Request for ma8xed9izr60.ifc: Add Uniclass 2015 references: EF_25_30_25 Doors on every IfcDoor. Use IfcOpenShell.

First a look at what the model holds.

```python
import ifcopenshell

model = ifcopenshell.open("ma8xed9izr60.ifc")
print(model.schema)
print("classifications:", [c.Name for c in model.by_type("IfcClassification")])
for ifc_class in ("IfcDoor", "IfcRoof", "IfcStair", "IfcWall", "IfcWindow"):
    print(ifc_class, len(model.by_type(ifc_class)))
```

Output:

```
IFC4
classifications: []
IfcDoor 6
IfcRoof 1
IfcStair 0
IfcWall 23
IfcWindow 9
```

```python
import ifcopenshell
import ifcopenshell.api.classification

model = ifcopenshell.open("ma8xed9izr60.ifc")

system = ifcopenshell.api.classification.add_classification(model, classification="Uniclass 2015")

codes = {
    "IfcDoor": ("EF_25_30_25", "Doors"),
}
for ifc_class, (code, name) in codes.items():
    products = model.by_type(ifc_class)
    ifcopenshell.api.classification.add_reference(
        model, products=products, classification=system, identification=code, name=name
    )
    print(code, len(products))

model.write("ma8xed9izr60_rev.ifc")
```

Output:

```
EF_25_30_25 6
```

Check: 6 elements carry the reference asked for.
